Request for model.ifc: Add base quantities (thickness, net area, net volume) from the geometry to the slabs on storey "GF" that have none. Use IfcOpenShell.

First a look at what the model holds.

```python
import ifcopenshell
import ifcopenshell.util.element
import ifcopenshell.util.unit

model = ifcopenshell.open("model.ifc")
print(model.schema)
for unit_type in ("LENGTHUNIT", "AREAUNIT", "VOLUMEUNIT"):
    print(unit_type, ifcopenshell.util.unit.calculate_unit_scale(model, unit_type))
storey = next(s for s in model.by_type("IfcBuildingStorey") if s.Name == "GF")
slabs = [e for e in ifcopenshell.util.element.get_decomposition(storey) if e.is_a("IfcSlab")]
for e in sorted(slabs, key=lambda e: e.id()):
    print(e.id(), e.is_a(), e.Name, list(ifcopenshell.util.element.get_psets(e, qtos_only=True)), sep=" | ")
```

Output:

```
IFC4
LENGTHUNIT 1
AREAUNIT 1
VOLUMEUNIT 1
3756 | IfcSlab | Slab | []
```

```python
import ifcopenshell
import ifcopenshell.api.pset
import ifcopenshell.geom
import ifcopenshell.util.element
import ifcopenshell.util.shape
import ifcopenshell.util.unit

model = ifcopenshell.open("model.ifc")
unit_scale = ifcopenshell.util.unit.calculate_unit_scale(model)
area_scale = ifcopenshell.util.unit.calculate_unit_scale(model, "AREAUNIT")
volume_scale = ifcopenshell.util.unit.calculate_unit_scale(model, "VOLUMEUNIT")
settings = ifcopenshell.geom.settings()

storey = next(s for s in model.by_type("IfcBuildingStorey") if s.Name == "GF")
slabs = [e for e in ifcopenshell.util.element.get_decomposition(storey) if e.is_a("IfcSlab")]

for e in sorted(slabs, key=lambda e: e.id()):
    if ifcopenshell.util.element.get_psets(e, qtos_only=True, should_inherit=False):
        continue
    # Geometry comes back in metres, in the element's own axes.
    shape = ifcopenshell.geom.create_shape(settings, e)
    values = {
        "Width": ifcopenshell.util.shape.get_z(shape.geometry) / unit_scale,
        "NetArea": ifcopenshell.util.shape.get_footprint_area(shape.geometry) / area_scale,
        "NetVolume": ifcopenshell.util.shape.get_volume(shape.geometry) / volume_scale,
    }
    qto = ifcopenshell.api.pset.add_qto(model, product=e, name="Qto_SlabBaseQuantities")
    ifcopenshell.api.pset.edit_qto(model, qto=qto, properties=values)
    print(e.id(), {k: round(v, 3) for k, v in values.items()})

model.write("model_rev.ifc")
```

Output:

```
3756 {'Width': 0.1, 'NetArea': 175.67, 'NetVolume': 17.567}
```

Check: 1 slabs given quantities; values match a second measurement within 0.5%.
